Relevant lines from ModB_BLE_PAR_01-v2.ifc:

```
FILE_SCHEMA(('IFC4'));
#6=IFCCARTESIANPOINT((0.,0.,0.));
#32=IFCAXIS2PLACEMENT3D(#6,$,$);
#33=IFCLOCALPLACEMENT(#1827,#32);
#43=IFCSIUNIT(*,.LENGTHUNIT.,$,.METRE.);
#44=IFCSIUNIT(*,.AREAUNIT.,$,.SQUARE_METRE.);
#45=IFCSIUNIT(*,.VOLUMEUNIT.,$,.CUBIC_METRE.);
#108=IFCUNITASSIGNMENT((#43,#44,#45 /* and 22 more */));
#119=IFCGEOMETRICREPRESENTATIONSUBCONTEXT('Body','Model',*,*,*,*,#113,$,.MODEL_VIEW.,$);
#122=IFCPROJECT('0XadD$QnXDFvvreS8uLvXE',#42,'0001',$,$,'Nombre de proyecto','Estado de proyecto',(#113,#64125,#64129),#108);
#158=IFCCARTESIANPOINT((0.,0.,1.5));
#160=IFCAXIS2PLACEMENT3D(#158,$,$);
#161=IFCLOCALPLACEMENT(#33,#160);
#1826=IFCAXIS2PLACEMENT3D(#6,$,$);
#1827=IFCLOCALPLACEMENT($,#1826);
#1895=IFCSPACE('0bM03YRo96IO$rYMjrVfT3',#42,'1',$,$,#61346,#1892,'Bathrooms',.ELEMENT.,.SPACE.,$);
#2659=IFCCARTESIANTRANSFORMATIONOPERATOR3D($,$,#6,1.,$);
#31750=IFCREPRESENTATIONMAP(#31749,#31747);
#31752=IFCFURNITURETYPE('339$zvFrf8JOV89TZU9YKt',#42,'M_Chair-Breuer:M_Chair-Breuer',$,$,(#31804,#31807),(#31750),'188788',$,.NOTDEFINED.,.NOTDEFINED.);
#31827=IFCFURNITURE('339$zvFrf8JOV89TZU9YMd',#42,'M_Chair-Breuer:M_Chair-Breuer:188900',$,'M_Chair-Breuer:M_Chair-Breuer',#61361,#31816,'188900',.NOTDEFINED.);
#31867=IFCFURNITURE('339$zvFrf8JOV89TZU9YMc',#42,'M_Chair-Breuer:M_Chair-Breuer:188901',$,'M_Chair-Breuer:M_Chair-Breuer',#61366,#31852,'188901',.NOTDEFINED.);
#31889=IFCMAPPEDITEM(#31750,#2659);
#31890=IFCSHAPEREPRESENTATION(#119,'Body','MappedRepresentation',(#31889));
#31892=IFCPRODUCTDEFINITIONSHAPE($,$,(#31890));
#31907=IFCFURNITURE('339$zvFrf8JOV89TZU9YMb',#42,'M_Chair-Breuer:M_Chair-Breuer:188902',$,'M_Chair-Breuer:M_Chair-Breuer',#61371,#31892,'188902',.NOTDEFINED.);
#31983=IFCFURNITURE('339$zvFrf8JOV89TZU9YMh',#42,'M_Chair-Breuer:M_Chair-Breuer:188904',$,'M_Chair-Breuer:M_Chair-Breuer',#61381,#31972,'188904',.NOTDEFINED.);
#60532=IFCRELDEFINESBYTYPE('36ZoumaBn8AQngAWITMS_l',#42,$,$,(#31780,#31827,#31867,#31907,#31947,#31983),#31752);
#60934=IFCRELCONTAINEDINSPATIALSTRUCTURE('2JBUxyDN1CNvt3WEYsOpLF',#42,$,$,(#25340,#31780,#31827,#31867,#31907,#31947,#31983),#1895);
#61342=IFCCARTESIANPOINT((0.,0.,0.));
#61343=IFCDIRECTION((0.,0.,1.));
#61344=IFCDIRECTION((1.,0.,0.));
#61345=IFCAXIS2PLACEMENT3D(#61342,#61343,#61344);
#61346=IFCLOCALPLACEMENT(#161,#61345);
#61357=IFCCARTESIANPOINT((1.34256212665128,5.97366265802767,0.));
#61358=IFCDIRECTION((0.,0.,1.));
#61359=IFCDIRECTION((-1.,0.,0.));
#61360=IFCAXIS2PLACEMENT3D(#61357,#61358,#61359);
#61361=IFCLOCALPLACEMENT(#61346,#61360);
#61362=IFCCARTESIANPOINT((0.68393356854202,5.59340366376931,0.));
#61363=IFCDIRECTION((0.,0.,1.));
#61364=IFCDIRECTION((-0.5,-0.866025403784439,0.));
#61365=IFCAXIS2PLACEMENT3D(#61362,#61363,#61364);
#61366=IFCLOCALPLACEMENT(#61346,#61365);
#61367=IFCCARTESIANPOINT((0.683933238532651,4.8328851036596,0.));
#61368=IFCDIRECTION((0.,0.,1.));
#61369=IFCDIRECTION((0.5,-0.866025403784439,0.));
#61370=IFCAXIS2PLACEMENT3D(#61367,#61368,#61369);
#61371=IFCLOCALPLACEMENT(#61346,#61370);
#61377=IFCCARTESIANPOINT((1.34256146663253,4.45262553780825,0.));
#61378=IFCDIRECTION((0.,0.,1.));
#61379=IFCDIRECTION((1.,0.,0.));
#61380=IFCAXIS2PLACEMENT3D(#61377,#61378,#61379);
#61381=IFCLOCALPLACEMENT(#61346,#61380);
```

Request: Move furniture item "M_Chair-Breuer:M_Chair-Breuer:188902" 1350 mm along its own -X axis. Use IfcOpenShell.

```python
import ifcopenshell
import ifcopenshell.api.geometry
import ifcopenshell.util.placement
import ifcopenshell.util.unit

model = ifcopenshell.open("ModB_BLE_PAR_01-v2.ifc")
unit_scale = ifcopenshell.util.unit.calculate_unit_scale(model)

item = model.by_id(31907)
matrix = ifcopenshell.util.placement.get_local_placement(item.ObjectPlacement)
matrix[:3, 3] -= matrix[:3, 0] * 1.35 / unit_scale
ifcopenshell.api.geometry.edit_object_placement(model, product=item, matrix=matrix, is_si=False)

print(ifcopenshell.util.placement.get_local_placement(item.ObjectPlacement).round(3) + 0.0)

model.write("ModB_BLE_PAR_01-v2_edited.ifc")
```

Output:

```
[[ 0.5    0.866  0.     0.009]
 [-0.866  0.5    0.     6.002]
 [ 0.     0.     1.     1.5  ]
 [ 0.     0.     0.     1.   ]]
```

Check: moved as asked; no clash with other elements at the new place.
